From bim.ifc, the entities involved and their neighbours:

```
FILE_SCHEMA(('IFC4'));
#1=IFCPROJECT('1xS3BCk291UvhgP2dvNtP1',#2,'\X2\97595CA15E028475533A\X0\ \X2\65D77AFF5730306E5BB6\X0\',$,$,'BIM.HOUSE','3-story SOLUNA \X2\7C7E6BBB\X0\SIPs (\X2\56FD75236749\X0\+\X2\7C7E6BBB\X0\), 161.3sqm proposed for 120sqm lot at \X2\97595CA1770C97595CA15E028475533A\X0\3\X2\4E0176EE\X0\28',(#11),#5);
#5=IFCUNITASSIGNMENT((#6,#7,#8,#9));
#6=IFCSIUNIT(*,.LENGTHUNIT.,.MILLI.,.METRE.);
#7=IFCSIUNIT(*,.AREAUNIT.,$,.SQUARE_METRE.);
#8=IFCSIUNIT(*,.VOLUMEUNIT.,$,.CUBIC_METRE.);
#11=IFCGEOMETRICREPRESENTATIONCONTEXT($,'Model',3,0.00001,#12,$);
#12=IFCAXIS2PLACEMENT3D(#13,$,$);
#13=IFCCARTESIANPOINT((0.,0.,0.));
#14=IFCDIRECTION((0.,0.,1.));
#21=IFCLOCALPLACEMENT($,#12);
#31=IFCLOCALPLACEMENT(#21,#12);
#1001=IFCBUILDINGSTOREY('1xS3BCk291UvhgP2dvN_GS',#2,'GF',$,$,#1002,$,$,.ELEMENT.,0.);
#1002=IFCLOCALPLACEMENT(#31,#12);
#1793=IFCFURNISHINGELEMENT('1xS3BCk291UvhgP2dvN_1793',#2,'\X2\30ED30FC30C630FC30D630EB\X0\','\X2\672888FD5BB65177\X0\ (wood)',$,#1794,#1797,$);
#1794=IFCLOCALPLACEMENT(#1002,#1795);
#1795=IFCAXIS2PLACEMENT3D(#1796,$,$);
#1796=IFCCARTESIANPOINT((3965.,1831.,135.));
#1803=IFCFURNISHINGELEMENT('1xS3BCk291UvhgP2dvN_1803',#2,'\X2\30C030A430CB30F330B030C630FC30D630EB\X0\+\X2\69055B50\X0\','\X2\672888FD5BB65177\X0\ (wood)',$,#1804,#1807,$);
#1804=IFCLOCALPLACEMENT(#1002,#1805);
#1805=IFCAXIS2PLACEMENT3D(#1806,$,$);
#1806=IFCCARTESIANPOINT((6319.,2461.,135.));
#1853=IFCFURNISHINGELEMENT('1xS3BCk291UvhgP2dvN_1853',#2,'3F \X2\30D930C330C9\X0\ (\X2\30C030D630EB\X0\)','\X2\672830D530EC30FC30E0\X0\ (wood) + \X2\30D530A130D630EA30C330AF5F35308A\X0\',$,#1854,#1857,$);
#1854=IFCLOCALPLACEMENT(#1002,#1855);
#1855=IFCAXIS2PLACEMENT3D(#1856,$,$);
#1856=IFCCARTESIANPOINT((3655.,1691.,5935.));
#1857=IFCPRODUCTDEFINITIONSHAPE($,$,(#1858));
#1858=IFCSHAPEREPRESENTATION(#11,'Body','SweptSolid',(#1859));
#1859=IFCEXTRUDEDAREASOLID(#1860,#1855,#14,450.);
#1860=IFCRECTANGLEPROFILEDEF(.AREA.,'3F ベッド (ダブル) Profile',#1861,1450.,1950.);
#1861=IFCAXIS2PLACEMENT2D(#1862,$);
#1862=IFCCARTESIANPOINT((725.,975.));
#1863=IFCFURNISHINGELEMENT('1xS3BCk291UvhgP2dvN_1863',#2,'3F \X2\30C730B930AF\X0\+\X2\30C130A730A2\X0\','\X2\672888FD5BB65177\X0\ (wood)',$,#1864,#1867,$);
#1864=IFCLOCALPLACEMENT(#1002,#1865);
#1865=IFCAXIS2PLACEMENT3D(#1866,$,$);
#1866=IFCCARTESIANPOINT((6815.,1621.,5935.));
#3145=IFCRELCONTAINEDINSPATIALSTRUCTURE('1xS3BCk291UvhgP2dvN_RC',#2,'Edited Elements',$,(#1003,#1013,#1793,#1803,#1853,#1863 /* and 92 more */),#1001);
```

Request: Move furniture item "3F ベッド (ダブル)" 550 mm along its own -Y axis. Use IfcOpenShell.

```python
import ifcopenshell
import ifcopenshell.api.geometry
import ifcopenshell.util.placement
import ifcopenshell.util.unit

model = ifcopenshell.open("bim.ifc")
unit_scale = ifcopenshell.util.unit.calculate_unit_scale(model)

item = model.by_id(1853)
matrix = ifcopenshell.util.placement.get_local_placement(item.ObjectPlacement)
matrix[:3, 3] -= matrix[:3, 1] * 0.55 / unit_scale
ifcopenshell.api.geometry.edit_object_placement(model, product=item, matrix=matrix, is_si=False)

print(ifcopenshell.util.placement.get_local_placement(item.ObjectPlacement).round(3) + 0.0)

model.write("bim_updated.ifc")
```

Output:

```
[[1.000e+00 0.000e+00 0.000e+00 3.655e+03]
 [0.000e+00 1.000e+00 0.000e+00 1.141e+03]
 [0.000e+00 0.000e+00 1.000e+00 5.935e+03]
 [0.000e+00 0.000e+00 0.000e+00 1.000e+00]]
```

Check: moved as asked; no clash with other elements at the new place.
